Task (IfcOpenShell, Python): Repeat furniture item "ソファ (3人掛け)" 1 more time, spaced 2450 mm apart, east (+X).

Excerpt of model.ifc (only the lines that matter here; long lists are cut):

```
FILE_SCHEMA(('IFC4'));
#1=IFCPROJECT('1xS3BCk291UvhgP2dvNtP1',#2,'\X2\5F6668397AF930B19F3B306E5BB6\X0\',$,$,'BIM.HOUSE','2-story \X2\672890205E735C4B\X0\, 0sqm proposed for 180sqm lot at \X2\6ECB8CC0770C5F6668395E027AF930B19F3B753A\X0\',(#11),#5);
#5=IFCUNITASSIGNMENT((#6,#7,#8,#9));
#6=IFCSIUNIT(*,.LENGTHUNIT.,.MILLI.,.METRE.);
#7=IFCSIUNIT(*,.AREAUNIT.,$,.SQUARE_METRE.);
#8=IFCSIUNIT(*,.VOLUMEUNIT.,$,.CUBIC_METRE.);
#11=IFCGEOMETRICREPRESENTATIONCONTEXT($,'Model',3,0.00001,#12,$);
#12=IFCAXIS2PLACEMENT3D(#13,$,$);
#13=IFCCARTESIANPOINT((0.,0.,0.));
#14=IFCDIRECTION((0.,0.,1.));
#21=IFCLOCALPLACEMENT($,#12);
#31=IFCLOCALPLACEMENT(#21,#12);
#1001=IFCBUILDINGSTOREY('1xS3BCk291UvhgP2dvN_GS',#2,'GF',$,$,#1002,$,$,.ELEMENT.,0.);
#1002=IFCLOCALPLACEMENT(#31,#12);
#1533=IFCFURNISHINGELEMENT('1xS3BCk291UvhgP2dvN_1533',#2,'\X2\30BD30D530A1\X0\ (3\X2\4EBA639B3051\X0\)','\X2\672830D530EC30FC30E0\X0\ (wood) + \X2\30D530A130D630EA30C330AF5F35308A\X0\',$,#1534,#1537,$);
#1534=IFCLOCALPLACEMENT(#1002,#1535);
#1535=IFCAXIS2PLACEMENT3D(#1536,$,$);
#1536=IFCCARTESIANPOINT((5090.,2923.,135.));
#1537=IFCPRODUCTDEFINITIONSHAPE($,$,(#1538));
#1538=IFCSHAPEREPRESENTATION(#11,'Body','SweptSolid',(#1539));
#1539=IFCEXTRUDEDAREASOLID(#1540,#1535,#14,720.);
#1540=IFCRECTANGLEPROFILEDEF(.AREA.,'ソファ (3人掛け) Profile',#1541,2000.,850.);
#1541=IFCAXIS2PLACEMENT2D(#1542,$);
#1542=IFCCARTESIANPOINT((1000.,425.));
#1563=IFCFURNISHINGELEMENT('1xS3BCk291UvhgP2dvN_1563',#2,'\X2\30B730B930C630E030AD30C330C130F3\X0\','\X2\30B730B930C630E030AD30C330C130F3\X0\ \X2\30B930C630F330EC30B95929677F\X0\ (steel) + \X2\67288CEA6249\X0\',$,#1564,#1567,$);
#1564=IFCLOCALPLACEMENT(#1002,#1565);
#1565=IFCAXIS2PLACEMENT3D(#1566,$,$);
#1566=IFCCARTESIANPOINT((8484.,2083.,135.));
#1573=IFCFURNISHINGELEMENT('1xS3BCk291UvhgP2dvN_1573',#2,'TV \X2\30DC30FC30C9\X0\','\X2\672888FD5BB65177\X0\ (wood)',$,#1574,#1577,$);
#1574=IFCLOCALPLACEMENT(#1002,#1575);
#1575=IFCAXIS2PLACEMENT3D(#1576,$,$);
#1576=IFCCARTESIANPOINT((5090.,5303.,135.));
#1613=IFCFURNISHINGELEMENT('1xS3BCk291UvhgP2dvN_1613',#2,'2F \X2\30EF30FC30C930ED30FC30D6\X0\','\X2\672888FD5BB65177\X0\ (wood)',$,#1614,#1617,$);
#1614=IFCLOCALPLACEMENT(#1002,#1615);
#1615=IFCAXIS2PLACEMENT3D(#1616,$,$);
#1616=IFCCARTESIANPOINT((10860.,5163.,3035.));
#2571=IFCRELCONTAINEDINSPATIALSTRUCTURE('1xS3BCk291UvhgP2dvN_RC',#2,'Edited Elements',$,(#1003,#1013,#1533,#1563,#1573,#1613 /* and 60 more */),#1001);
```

```python
import numpy as np
import ifcopenshell
import ifcopenshell.api.geometry
import ifcopenshell.api.root
import ifcopenshell.util.element
import ifcopenshell.util.placement

model = ifcopenshell.open("model.ifc")


def reuse_history(source, copy):
    """copy_class also copies each property set's owner history, people and application; keep the originals."""
    for rel in copy.IsDefinedBy:
        if rel.is_a("IfcRelDefinesByProperties") and (history := rel.RelatingPropertyDefinition.OwnerHistory):
            rel.RelatingPropertyDefinition.OwnerHistory = source.OwnerHistory
            ifcopenshell.util.element.remove_deep2(model, history)


source = model.by_id(1533)
base = ifcopenshell.util.placement.get_local_placement(source.ObjectPlacement)
step = np.array([1.0, 0.0, 0.0]) * 2450.0

for i in range(1, 2):
    copy = ifcopenshell.api.root.copy_class(model, product=source)
    copy.Representation = ifcopenshell.util.element.copy_deep(
        model, source.Representation, exclude=["IfcGeometricRepresentationContext", "IfcRepresentationMap"]
    )
    reuse_history(source, copy)
    matrix = base.copy()
    matrix[:3, 3] += i * step
    print("added at", matrix[:3, 3].round(3) + 0.0)
    ifcopenshell.api.geometry.edit_object_placement(model, product=copy, matrix=matrix, is_si=False)

model.write("model_updated.ifc")
```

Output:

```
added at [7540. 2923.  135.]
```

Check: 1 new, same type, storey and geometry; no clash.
